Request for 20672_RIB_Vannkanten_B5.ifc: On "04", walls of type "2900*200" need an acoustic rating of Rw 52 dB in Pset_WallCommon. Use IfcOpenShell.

First a look at what the model holds.

```python
import ifcopenshell
import ifcopenshell.util.element

model = ifcopenshell.open("20672_RIB_Vannkanten_B5.ifc")
print(model.schema)
storey = next(s for s in model.by_type("IfcBuildingStorey") if s.Name == "04")
walls = [e for e in ifcopenshell.util.element.get_decomposition(storey) if e.is_a("IfcWall")]
seen = {}
for e in walls:
    element_type = ifcopenshell.util.element.get_type(e)
    key = (element_type.Name if element_type != e and element_type else None, ifcopenshell.util.element.get_pset(e, "Pset_WallCommon", "AcousticRating"))
    seen[key] = seen.get(key, 0) + 1
for (name, value), count in sorted(seen.items(), key=str):
    print(count, "x", name, "|", value)
```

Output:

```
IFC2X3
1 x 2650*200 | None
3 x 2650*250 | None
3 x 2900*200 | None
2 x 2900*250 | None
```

```python
import ifcopenshell
import ifcopenshell.api.pset
import ifcopenshell.util.element

model = ifcopenshell.open("20672_RIB_Vannkanten_B5.ifc")

storey = next(s for s in model.by_type("IfcBuildingStorey") if s.Name == "04")
walls = [e for e in ifcopenshell.util.element.get_decomposition(storey) if e.is_a("IfcWall")]

count = 0
for e in walls:
    element_type = ifcopenshell.util.element.get_type(e)
    if element_type in (None, e) or element_type.Name != "2900*200":
        continue
    # add_pset returns the element's existing set when there is one.
    pset = ifcopenshell.api.pset.add_pset(model, product=e, name="Pset_WallCommon")
    ifcopenshell.api.pset.edit_pset(model, pset=pset, properties={"AcousticRating": "Rw 52 dB"})
    count += 1

print(count, "walls updated")

model.write("20672_RIB_Vannkanten_B5_updated.ifc")
```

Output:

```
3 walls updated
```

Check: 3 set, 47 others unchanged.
